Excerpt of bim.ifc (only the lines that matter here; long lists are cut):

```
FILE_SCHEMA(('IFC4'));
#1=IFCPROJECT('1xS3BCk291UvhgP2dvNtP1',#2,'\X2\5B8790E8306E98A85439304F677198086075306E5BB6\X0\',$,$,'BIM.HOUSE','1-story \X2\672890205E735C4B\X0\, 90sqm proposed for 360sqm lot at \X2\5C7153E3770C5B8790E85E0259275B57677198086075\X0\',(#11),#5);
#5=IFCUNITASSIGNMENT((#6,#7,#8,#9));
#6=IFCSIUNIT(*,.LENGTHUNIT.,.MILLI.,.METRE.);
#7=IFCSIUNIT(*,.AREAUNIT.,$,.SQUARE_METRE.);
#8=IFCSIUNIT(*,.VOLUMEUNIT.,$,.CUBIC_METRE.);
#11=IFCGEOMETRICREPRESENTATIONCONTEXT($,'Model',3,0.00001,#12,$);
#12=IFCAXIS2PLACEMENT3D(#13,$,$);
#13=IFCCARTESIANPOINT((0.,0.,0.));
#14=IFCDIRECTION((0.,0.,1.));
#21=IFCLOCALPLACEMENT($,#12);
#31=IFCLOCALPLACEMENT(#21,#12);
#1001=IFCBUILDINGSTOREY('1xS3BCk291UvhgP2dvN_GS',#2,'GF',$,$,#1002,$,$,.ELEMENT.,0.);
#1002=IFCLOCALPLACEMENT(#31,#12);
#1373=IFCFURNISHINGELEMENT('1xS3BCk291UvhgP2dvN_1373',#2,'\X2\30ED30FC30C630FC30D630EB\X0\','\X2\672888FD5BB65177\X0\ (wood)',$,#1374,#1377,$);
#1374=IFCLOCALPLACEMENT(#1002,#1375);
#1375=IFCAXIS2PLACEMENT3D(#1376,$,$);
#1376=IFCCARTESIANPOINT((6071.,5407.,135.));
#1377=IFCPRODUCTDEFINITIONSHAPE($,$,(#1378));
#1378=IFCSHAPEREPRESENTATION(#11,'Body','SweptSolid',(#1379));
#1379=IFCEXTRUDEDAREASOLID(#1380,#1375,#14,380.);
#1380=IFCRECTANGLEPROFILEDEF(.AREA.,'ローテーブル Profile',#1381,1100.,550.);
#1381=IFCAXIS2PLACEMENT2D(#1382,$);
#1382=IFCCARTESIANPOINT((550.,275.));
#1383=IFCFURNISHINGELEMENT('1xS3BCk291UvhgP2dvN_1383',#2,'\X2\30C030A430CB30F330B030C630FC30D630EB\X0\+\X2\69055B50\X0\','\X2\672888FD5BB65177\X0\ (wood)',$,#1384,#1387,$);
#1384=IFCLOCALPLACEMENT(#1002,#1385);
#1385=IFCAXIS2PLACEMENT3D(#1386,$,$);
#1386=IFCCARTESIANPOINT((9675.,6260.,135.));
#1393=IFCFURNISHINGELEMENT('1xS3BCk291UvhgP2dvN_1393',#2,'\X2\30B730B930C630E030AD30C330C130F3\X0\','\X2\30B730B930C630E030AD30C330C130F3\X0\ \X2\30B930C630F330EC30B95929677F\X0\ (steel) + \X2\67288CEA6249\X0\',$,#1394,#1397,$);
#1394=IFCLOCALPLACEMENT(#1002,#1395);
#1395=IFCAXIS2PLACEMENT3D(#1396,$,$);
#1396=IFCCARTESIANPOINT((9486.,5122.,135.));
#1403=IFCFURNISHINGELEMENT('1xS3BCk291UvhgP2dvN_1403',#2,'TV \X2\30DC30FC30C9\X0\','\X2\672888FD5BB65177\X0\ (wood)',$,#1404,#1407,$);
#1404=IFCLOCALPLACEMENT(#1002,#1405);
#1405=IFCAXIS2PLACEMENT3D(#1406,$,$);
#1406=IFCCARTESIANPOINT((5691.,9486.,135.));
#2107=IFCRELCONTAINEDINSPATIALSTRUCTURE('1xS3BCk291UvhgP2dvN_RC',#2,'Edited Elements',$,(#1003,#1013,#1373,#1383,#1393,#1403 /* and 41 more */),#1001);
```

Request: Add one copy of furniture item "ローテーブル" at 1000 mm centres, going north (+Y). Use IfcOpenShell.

```python
import numpy as np
import ifcopenshell
import ifcopenshell.api.geometry
import ifcopenshell.api.root
import ifcopenshell.util.element
import ifcopenshell.util.placement

model = ifcopenshell.open("bim.ifc")


def reuse_history(source, copy):
    """copy_class also copies each property set's owner history, people and application; keep the originals."""
    for rel in copy.IsDefinedBy:
        if rel.is_a("IfcRelDefinesByProperties") and (history := rel.RelatingPropertyDefinition.OwnerHistory):
            rel.RelatingPropertyDefinition.OwnerHistory = source.OwnerHistory
            ifcopenshell.util.element.remove_deep2(model, history)


source = model.by_id(1373)
base = ifcopenshell.util.placement.get_local_placement(source.ObjectPlacement)
step = np.array([0.0, 1.0, 0.0]) * 1000.0

for i in range(1, 2):
    copy = ifcopenshell.api.root.copy_class(model, product=source)
    copy.Representation = ifcopenshell.util.element.copy_deep(
        model, source.Representation, exclude=["IfcGeometricRepresentationContext", "IfcRepresentationMap"]
    )
    reuse_history(source, copy)
    matrix = base.copy()
    matrix[:3, 3] += i * step
    print("added at", matrix[:3, 3].round(3) + 0.0)
    ifcopenshell.api.geometry.edit_object_placement(model, product=copy, matrix=matrix, is_si=False)

model.write("bim-out.ifc")
```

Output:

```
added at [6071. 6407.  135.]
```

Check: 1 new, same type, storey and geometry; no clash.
